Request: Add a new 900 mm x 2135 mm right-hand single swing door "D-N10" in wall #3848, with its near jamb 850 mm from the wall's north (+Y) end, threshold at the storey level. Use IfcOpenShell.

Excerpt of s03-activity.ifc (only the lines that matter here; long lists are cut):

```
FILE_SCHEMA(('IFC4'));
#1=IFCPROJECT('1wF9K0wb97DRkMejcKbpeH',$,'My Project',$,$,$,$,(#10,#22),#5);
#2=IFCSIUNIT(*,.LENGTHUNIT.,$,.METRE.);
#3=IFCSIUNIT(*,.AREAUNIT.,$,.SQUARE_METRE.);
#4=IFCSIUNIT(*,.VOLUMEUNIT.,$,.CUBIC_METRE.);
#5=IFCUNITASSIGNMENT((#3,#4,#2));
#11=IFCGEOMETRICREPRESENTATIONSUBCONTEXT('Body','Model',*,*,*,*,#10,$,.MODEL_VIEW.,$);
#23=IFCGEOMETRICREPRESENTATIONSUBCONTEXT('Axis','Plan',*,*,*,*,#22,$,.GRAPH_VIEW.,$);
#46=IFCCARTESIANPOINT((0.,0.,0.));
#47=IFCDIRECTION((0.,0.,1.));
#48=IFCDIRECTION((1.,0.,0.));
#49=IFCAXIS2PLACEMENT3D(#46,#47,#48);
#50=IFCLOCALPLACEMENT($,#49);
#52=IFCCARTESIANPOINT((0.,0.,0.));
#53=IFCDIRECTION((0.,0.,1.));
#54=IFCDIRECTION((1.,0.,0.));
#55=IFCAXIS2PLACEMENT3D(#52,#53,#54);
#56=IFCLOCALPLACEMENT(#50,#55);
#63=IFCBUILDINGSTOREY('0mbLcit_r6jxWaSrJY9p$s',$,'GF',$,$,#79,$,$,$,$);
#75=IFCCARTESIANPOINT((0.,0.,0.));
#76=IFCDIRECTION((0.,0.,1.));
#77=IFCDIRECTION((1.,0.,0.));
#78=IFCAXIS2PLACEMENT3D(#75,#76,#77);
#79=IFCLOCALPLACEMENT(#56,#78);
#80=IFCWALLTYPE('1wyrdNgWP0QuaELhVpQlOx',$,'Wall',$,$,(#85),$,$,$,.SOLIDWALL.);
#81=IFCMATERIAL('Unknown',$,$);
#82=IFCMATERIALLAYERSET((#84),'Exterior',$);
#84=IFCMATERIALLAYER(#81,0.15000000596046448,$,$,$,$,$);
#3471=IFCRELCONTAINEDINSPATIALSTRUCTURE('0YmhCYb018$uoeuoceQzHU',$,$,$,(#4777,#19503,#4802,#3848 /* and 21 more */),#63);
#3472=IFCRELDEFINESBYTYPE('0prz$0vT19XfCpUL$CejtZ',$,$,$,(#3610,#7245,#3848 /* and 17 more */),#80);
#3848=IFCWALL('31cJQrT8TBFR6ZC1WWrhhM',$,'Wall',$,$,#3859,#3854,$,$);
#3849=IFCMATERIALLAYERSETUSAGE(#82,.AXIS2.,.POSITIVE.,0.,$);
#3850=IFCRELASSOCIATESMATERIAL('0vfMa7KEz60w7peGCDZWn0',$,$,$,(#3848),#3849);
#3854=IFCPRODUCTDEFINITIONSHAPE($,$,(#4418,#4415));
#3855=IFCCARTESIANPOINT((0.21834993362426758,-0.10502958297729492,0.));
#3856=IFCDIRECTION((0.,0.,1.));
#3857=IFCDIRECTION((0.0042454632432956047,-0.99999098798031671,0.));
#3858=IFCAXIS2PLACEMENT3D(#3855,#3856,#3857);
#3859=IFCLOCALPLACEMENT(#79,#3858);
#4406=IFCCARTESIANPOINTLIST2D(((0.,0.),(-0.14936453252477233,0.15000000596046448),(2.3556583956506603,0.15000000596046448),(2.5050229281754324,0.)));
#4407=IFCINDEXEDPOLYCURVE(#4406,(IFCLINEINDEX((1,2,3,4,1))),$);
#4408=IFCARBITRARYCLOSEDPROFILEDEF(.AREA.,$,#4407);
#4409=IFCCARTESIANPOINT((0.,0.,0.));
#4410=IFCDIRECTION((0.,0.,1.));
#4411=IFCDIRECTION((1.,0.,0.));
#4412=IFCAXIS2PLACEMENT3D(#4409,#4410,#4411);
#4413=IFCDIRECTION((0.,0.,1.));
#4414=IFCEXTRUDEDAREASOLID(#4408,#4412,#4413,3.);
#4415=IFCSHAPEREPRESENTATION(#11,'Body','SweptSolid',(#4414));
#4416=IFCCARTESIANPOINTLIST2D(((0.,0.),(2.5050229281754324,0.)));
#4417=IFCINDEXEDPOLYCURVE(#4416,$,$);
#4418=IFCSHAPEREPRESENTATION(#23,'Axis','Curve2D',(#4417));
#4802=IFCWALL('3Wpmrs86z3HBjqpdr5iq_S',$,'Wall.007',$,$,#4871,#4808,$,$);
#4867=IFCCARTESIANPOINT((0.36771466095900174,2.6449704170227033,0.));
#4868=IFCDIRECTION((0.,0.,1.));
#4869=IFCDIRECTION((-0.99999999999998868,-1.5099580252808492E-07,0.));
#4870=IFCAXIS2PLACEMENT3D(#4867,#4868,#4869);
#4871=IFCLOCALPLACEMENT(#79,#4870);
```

```python
import numpy as np
import ifcopenshell
import ifcopenshell.api.feature
import ifcopenshell.api.geometry
import ifcopenshell.api.root
import ifcopenshell.api.spatial
import ifcopenshell.geom
import ifcopenshell.util.element
import ifcopenshell.util.placement
import ifcopenshell.util.representation
import ifcopenshell.util.shape
import ifcopenshell.util.unit

model = ifcopenshell.open("s03-activity.ifc")
unit_scale = ifcopenshell.util.unit.calculate_unit_scale(model)
settings = ifcopenshell.geom.settings()


def volume(element):
    """Net volume in cubic metres, openings subtracted."""
    shape = ifcopenshell.geom.create_shape(settings, element)
    return ifcopenshell.util.shape.get_volume(shape.geometry)


wall = model.by_id(3848)
storey = ifcopenshell.util.element.get_container(wall, ifc_class="IfcBuildingStorey")
context = ifcopenshell.util.representation.get_context(model, "Model", "Body", "MODEL_VIEW")
before = volume(wall)

width, height, from_end, sill = 0.9, 2.135, 0.85, 0.0  # metres

# The wall runs along its own X axis, and the end named is its -X end.
wall_shape = ifcopenshell.geom.create_shape(settings, wall)
x, y, z = ifcopenshell.util.shape.get_vertices(wall_shape.geometry).T
start = x.min() + from_end
face, thickness = float(y.min()), float(y.max() - y.min())
wall_matrix = ifcopenshell.util.placement.get_local_placement(wall.ObjectPlacement)
level = ifcopenshell.util.placement.get_local_placement(storey.ObjectPlacement)[2, 3]


def in_wall(x, y):
    """Placement at x, y metres in the wall's axes, at sill height."""
    matrix = wall_matrix.copy()
    matrix[:, 3] = wall_matrix @ np.array([x / unit_scale, y / unit_scale, 0.0, 1.0])
    matrix[2, 3] = level + sill / unit_scale
    return matrix


# Opening: a box that overshoots both wall faces by 50 mm.
opening = ifcopenshell.api.root.create_entity(model, ifc_class="IfcOpeningElement", predefined_type="OPENING")
box = ifcopenshell.api.geometry.add_wall_representation(
    model, context=context, length=width, height=height, thickness=thickness + 0.1
)
ifcopenshell.api.geometry.assign_representation(model, product=opening, representation=box)
ifcopenshell.api.geometry.edit_object_placement(model, product=opening, matrix=in_wall(start, face - 0.05), is_si=False)
ifcopenshell.api.feature.add_feature(model, feature=opening, element=wall)

door = ifcopenshell.api.root.create_entity(model, ifc_class="IfcDoor", name="D-N10", predefined_type="DOOR")
door.OverallWidth, door.OverallHeight = width / unit_scale, height / unit_scale
door.OperationType = "SINGLE_SWING_RIGHT"
body = ifcopenshell.api.geometry.add_door_representation(
    model,
    context=context,
    overall_width=door.OverallWidth,
    overall_height=door.OverallHeight,
    operation_type="SINGLE_SWING_RIGHT",
    lining_properties={"LiningDepth": thickness / unit_scale, "ThresholdDepth": thickness / unit_scale},
)
ifcopenshell.api.geometry.assign_representation(model, product=door, representation=body)
ifcopenshell.api.spatial.assign_container(model, products=[door], relating_structure=storey)
ifcopenshell.api.feature.add_filling(model, opening=opening, element=door)

# The lining spans the wall, so the door starts at the wall face.
ifcopenshell.api.geometry.edit_object_placement(model, product=door, matrix=in_wall(start, face), is_si=False)

after = volume(wall)

print(f"wall volume {before:.3f} -> {after:.3f} m3")

model.write("s03-activity_updated.ifc")
```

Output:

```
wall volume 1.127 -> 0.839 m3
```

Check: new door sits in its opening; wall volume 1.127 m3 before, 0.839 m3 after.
